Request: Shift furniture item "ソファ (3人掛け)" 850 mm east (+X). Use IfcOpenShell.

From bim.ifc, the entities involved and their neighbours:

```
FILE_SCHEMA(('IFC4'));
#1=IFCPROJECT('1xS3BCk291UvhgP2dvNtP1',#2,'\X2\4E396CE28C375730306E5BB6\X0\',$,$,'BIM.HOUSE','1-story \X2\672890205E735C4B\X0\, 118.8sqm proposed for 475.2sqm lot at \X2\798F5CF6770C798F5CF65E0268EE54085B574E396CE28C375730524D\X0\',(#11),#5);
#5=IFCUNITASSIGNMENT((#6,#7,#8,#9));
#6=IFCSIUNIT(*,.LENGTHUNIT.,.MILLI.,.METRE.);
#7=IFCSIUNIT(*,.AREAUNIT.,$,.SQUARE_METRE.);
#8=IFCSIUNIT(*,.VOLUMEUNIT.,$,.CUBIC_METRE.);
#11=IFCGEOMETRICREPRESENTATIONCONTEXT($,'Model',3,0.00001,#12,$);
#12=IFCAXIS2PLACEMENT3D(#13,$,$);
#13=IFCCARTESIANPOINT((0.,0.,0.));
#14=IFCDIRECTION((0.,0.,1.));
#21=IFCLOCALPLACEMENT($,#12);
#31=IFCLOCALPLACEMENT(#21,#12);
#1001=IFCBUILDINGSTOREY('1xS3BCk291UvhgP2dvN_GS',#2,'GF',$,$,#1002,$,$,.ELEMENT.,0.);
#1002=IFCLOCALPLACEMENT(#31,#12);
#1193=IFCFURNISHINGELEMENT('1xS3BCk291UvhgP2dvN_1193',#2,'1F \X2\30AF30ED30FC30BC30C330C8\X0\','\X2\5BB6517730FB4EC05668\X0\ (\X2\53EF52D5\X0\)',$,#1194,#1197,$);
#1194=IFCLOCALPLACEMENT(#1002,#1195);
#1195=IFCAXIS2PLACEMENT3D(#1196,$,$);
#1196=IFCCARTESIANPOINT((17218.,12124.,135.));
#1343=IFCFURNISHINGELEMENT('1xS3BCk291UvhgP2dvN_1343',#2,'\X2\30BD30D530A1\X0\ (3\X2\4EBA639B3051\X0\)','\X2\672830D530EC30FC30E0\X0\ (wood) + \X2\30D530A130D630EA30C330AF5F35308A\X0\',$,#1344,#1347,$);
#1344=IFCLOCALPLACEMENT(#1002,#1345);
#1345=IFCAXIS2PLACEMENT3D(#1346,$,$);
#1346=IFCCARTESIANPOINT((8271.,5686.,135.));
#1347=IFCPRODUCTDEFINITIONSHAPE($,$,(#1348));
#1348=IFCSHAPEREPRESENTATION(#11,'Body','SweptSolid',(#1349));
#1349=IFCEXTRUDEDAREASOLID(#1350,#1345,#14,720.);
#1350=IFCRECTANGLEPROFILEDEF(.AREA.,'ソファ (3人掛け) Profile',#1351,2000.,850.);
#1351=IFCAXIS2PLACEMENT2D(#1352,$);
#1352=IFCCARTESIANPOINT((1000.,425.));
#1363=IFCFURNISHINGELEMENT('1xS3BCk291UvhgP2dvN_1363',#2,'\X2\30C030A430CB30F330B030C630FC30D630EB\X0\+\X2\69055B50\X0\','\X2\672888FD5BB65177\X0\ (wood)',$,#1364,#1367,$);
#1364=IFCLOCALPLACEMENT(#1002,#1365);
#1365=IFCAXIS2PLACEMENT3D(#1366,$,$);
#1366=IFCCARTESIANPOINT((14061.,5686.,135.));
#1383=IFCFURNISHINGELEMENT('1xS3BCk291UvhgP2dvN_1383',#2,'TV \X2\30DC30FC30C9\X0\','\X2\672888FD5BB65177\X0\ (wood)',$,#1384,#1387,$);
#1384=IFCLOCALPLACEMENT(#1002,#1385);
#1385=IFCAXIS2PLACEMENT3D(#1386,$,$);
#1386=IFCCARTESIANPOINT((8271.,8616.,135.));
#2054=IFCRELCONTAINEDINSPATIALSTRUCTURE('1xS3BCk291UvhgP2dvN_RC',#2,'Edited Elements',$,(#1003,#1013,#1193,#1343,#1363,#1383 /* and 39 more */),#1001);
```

```python
import ifcopenshell
import ifcopenshell.api.geometry
import ifcopenshell.util.placement

model = ifcopenshell.open("bim.ifc")

item = model.by_guid("1xS3BCk291UvhgP2dvN_1343")
matrix = ifcopenshell.util.placement.get_local_placement(item.ObjectPlacement)
matrix[0, 3] += 850.0
ifcopenshell.api.geometry.edit_object_placement(model, product=item, matrix=matrix, is_si=False)

print(ifcopenshell.util.placement.get_local_placement(item.ObjectPlacement).round(3) + 0.0)

model.write("bim_updated.ifc")
```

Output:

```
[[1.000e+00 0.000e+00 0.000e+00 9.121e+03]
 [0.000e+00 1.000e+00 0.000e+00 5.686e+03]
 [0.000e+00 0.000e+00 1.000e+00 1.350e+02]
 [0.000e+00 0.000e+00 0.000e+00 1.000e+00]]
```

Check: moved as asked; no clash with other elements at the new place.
